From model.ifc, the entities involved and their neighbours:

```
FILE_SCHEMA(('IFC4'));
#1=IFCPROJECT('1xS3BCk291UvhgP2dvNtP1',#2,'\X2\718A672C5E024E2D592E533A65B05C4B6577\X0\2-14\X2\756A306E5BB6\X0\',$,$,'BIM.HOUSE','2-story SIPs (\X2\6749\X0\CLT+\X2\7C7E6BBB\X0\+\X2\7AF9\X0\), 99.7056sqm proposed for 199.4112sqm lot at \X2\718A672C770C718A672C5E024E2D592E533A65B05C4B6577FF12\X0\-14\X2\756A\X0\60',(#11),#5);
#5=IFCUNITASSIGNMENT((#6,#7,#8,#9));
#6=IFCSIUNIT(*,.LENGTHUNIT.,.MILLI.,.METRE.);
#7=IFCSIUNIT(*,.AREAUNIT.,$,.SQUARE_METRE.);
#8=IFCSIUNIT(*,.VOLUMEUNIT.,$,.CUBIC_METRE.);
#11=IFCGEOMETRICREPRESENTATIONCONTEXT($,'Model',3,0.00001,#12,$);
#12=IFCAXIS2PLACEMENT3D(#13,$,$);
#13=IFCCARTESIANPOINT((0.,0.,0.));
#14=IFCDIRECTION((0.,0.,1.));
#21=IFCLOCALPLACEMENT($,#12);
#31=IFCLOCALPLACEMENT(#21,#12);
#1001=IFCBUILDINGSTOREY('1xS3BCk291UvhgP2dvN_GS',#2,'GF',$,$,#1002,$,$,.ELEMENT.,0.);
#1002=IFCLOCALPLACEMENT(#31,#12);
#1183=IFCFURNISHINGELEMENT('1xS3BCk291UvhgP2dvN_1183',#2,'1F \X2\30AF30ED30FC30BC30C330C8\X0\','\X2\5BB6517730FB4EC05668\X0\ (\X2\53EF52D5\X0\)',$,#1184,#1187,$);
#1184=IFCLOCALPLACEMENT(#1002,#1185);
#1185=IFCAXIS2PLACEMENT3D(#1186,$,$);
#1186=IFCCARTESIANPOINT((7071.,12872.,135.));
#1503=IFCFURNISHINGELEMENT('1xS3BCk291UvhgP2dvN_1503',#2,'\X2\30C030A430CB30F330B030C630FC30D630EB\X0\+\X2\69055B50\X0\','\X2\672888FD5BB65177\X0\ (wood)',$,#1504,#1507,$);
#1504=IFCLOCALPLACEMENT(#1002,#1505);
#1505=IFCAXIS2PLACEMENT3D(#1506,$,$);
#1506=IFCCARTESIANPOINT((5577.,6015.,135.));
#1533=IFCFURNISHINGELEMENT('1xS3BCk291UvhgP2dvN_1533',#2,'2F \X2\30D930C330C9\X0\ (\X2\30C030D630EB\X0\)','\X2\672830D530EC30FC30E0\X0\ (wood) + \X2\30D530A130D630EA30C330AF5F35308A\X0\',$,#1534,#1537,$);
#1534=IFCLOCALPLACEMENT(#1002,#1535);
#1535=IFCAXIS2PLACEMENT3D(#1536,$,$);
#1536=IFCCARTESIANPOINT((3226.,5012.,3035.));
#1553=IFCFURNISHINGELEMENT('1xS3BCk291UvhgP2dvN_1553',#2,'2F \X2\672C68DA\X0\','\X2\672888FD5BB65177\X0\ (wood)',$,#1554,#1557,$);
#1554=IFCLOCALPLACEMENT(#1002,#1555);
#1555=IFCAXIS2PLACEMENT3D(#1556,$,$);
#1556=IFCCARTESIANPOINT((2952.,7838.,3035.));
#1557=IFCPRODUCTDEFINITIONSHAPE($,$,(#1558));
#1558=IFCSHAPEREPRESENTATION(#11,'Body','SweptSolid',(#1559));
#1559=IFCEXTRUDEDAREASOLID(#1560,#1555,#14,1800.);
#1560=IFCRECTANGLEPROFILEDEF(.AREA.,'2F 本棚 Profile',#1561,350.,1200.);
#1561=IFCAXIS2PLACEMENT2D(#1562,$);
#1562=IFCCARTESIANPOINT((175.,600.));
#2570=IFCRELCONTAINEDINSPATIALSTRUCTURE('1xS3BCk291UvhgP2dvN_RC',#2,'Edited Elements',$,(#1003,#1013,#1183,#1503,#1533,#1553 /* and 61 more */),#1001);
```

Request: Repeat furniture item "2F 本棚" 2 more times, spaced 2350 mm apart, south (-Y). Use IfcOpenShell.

```python
import numpy as np
import ifcopenshell
import ifcopenshell.api.geometry
import ifcopenshell.api.root
import ifcopenshell.util.element
import ifcopenshell.util.placement

model = ifcopenshell.open("model.ifc")


def reuse_history(source, copy):
    """copy_class also copies each property set's owner history, people and application; keep the originals."""
    for rel in copy.IsDefinedBy:
        if rel.is_a("IfcRelDefinesByProperties") and (history := rel.RelatingPropertyDefinition.OwnerHistory):
            rel.RelatingPropertyDefinition.OwnerHistory = source.OwnerHistory
            ifcopenshell.util.element.remove_deep2(model, history)


source = model.by_guid("1xS3BCk291UvhgP2dvN_1553")
base = ifcopenshell.util.placement.get_local_placement(source.ObjectPlacement)
step = np.array([0.0, -1.0, 0.0]) * 2350.0

for i in range(1, 3):
    copy = ifcopenshell.api.root.copy_class(model, product=source)
    copy.Representation = ifcopenshell.util.element.copy_deep(
        model, source.Representation, exclude=["IfcGeometricRepresentationContext", "IfcRepresentationMap"]
    )
    reuse_history(source, copy)
    matrix = base.copy()
    matrix[:3, 3] += i * step
    print("added at", matrix[:3, 3].round(3) + 0.0)
    ifcopenshell.api.geometry.edit_object_placement(model, product=copy, matrix=matrix, is_si=False)

model.write("model-out.ifc")
```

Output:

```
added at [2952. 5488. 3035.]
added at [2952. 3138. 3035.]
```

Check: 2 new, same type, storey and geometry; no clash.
